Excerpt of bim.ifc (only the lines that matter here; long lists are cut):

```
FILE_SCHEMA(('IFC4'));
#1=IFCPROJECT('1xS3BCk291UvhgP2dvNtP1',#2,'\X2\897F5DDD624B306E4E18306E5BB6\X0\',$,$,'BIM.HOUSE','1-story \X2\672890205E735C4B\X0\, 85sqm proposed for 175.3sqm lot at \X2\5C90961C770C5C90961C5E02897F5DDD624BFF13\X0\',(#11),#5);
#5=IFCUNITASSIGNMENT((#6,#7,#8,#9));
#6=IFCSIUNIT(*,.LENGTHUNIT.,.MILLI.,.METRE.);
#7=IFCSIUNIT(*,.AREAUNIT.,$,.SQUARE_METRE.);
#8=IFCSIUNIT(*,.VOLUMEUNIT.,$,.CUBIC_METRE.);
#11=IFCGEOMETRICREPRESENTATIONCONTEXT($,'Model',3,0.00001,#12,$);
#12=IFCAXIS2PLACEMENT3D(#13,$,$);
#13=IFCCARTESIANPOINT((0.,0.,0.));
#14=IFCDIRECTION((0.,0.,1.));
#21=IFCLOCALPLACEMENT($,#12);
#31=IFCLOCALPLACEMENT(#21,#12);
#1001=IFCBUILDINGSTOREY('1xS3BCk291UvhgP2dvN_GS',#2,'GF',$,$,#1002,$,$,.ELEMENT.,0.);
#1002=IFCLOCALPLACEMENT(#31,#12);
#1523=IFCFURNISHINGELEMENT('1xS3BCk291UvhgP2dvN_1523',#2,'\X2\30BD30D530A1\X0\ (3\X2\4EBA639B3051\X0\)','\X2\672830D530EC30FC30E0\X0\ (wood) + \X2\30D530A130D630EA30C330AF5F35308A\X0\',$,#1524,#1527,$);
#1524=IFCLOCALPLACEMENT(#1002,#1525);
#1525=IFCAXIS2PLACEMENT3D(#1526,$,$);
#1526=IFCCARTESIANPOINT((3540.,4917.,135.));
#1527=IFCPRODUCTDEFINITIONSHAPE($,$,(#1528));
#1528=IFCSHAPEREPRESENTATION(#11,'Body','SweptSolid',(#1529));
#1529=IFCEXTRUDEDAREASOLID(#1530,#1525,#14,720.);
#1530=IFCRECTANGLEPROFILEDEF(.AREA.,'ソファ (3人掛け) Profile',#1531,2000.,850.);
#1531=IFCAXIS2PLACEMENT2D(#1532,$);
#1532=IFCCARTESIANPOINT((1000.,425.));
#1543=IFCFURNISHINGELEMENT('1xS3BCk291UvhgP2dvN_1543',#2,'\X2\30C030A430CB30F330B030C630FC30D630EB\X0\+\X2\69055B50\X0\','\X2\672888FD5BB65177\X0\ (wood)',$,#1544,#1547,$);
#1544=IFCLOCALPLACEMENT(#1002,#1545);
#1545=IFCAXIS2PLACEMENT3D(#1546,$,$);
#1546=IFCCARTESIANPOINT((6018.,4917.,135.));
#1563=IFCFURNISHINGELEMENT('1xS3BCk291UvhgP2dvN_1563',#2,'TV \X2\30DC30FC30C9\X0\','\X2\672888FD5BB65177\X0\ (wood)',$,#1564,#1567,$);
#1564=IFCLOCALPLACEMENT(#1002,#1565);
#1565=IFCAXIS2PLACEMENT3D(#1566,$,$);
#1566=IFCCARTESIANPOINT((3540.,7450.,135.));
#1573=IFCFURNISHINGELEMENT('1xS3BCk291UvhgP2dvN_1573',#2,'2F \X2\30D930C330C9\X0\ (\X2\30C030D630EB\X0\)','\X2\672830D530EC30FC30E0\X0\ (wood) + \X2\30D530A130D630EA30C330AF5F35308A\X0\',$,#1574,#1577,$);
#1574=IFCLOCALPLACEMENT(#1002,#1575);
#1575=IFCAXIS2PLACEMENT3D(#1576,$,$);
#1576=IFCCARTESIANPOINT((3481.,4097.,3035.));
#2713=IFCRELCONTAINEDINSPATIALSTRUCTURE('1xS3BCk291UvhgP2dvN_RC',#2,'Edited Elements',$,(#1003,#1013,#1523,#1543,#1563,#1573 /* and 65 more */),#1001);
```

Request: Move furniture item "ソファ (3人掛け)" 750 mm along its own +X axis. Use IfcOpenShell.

```python
import ifcopenshell
import ifcopenshell.api.geometry
import ifcopenshell.util.placement
import ifcopenshell.util.unit

model = ifcopenshell.open("bim.ifc")
unit_scale = ifcopenshell.util.unit.calculate_unit_scale(model)

item = model.by_guid("1xS3BCk291UvhgP2dvN_1523")
matrix = ifcopenshell.util.placement.get_local_placement(item.ObjectPlacement)
matrix[:3, 3] += matrix[:3, 0] * 0.75 / unit_scale
ifcopenshell.api.geometry.edit_object_placement(model, product=item, matrix=matrix, is_si=False)

print(ifcopenshell.util.placement.get_local_placement(item.ObjectPlacement).round(3) + 0.0)

model.write("bim_v2.ifc")
```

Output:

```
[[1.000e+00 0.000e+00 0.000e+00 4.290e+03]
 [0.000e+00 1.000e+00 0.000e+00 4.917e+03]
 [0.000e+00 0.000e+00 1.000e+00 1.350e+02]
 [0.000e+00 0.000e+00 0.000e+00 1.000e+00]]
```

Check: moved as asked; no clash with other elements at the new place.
